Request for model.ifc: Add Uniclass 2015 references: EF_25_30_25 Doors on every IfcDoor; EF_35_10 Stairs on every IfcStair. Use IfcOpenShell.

First a look at what the model holds.

```python
import ifcopenshell

model = ifcopenshell.open("model.ifc")
print(model.schema)
print("classifications:", [c.Name for c in model.by_type("IfcClassification")])
for ifc_class in ("IfcDoor", "IfcRoof", "IfcStair", "IfcWall", "IfcWindow"):
    print(ifc_class, len(model.by_type(ifc_class)))
```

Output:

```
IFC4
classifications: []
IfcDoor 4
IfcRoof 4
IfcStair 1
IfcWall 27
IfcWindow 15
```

```python
import ifcopenshell
import ifcopenshell.api.classification

model = ifcopenshell.open("model.ifc")

system = ifcopenshell.api.classification.add_classification(model, classification="Uniclass 2015")

codes = {
    "IfcDoor": ("EF_25_30_25", "Doors"),
    "IfcStair": ("EF_35_10", "Stairs"),
}
for ifc_class, (code, name) in codes.items():
    products = model.by_type(ifc_class)
    ifcopenshell.api.classification.add_reference(
        model, products=products, classification=system, identification=code, name=name
    )
    print(code, len(products))

model.write("model-out.ifc")
```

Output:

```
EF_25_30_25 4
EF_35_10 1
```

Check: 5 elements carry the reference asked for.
